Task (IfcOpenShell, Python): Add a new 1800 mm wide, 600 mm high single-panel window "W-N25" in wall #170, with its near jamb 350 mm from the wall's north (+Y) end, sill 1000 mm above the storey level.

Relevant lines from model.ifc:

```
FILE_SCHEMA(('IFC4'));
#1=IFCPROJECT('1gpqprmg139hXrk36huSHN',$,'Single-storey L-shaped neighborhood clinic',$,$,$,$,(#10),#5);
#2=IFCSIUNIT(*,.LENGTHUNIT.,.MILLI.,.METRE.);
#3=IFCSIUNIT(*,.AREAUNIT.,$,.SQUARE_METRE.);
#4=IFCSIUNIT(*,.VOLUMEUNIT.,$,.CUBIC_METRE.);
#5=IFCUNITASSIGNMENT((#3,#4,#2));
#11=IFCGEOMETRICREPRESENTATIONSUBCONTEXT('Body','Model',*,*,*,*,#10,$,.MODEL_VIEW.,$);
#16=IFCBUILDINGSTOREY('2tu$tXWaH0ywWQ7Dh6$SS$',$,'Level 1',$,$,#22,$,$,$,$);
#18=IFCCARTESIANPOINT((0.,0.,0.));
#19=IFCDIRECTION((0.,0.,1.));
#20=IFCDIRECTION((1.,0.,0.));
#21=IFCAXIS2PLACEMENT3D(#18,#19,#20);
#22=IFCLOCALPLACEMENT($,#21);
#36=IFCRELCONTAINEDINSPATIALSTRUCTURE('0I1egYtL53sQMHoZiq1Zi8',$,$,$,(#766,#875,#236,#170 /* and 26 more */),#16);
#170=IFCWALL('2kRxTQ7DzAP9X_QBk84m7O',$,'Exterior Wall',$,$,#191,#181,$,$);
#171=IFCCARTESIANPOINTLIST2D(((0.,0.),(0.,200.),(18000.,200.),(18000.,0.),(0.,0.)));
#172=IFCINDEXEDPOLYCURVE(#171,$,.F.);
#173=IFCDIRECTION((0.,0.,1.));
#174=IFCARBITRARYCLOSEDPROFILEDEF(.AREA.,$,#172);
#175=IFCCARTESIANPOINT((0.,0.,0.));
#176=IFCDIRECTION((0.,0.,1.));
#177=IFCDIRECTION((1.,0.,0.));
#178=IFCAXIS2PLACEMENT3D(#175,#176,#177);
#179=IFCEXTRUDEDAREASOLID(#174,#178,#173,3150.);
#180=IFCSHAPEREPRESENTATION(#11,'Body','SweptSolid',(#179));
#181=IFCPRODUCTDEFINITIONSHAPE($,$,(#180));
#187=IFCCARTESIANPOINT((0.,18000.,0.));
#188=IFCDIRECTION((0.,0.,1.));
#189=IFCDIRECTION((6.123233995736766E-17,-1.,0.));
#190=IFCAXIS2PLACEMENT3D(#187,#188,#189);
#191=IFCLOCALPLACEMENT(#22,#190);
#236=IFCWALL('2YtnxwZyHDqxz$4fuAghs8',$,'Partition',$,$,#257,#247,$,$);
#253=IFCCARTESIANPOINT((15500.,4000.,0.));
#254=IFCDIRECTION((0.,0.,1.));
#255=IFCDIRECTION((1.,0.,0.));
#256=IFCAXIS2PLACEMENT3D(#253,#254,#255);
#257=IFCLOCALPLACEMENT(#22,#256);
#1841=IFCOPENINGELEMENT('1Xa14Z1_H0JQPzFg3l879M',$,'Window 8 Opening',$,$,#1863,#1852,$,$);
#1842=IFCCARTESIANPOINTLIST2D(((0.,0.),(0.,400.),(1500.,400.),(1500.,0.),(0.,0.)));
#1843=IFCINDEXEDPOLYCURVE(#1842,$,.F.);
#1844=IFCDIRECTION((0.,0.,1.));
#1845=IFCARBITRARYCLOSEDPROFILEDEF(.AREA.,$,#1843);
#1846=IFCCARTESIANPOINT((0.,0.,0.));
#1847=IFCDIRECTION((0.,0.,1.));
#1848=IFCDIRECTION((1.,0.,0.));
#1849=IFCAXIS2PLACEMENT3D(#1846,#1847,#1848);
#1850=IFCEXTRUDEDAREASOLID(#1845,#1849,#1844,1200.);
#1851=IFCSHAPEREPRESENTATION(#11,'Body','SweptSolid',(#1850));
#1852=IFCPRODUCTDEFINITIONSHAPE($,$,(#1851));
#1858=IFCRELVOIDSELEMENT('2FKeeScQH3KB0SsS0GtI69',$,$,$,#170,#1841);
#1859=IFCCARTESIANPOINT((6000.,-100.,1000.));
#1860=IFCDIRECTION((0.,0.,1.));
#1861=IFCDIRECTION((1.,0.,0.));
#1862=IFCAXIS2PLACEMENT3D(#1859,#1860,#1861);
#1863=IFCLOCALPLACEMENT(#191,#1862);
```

```python
import numpy as np
import ifcopenshell
import ifcopenshell.api.feature
import ifcopenshell.api.geometry
import ifcopenshell.api.root
import ifcopenshell.api.spatial
import ifcopenshell.geom
import ifcopenshell.util.element
import ifcopenshell.util.placement
import ifcopenshell.util.representation
import ifcopenshell.util.shape
import ifcopenshell.util.unit

model = ifcopenshell.open("model.ifc")
unit_scale = ifcopenshell.util.unit.calculate_unit_scale(model)
settings = ifcopenshell.geom.settings()


def volume(element):
    """Net volume in cubic metres, openings subtracted."""
    shape = ifcopenshell.geom.create_shape(settings, element)
    return ifcopenshell.util.shape.get_volume(shape.geometry)


wall = model.by_guid("2kRxTQ7DzAP9X_QBk84m7O")
storey = ifcopenshell.util.element.get_container(wall, ifc_class="IfcBuildingStorey")
context = ifcopenshell.util.representation.get_context(model, "Model", "Body", "MODEL_VIEW")
before = volume(wall)

width, height, from_end, sill = 1.8, 0.6, 0.35, 1  # metres

# The wall runs along its own X axis, and the end named is its -X end.
wall_shape = ifcopenshell.geom.create_shape(settings, wall)
x, y, z = ifcopenshell.util.shape.get_vertices(wall_shape.geometry).T
start = x.min() + from_end
face, thickness = float(y.min()), float(y.max() - y.min())
wall_matrix = ifcopenshell.util.placement.get_local_placement(wall.ObjectPlacement)
level = ifcopenshell.util.placement.get_local_placement(storey.ObjectPlacement)[2, 3]


def in_wall(x, y):
    """Placement at x, y metres in the wall's axes, at sill height."""
    matrix = wall_matrix.copy()
    matrix[:, 3] = wall_matrix @ np.array([x / unit_scale, y / unit_scale, 0.0, 1.0])
    matrix[2, 3] = level + sill / unit_scale
    return matrix


# Opening: a box that overshoots both wall faces by 50 mm.
opening = ifcopenshell.api.root.create_entity(model, ifc_class="IfcOpeningElement", predefined_type="OPENING")
box = ifcopenshell.api.geometry.add_wall_representation(
    model, context=context, length=width, height=height, thickness=thickness + 0.1
)
ifcopenshell.api.geometry.assign_representation(model, product=opening, representation=box)
ifcopenshell.api.geometry.edit_object_placement(model, product=opening, matrix=in_wall(start, face - 0.05), is_si=False)
ifcopenshell.api.feature.add_feature(model, feature=opening, element=wall)

window = ifcopenshell.api.root.create_entity(model, ifc_class="IfcWindow", name="W-N25", predefined_type="WINDOW")
window.OverallWidth, window.OverallHeight = width / unit_scale, height / unit_scale
window.PartitioningType = "SINGLE_PANEL"
body = ifcopenshell.api.geometry.add_window_representation(
    model,
    context=context,
    overall_width=window.OverallWidth,
    overall_height=window.OverallHeight,
    partition_type="SINGLE_PANEL",
)
ifcopenshell.api.geometry.assign_representation(model, product=window, representation=body)
ifcopenshell.api.spatial.assign_container(model, products=[window], relating_structure=storey)
ifcopenshell.api.feature.add_filling(model, opening=opening, element=window)

# Centre the window in the wall's thickness.
ifcopenshell.api.geometry.edit_object_placement(model, product=window, matrix=in_wall(start, face), is_si=False)
window_shape = ifcopenshell.geom.create_shape(settings, window)
depth = ifcopenshell.util.shape.get_vertices(window_shape.geometry)[:, 1]
offset = face + thickness / 2 - (depth.min() + depth.max()) / 2
ifcopenshell.api.geometry.edit_object_placement(model, product=window, matrix=in_wall(start, offset), is_si=False)

after = volume(wall)

print(f"wall volume {before:.3f} -> {after:.3f} m3")

model.write("model_rev.ifc")
```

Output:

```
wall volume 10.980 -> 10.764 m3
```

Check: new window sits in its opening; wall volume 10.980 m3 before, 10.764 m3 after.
